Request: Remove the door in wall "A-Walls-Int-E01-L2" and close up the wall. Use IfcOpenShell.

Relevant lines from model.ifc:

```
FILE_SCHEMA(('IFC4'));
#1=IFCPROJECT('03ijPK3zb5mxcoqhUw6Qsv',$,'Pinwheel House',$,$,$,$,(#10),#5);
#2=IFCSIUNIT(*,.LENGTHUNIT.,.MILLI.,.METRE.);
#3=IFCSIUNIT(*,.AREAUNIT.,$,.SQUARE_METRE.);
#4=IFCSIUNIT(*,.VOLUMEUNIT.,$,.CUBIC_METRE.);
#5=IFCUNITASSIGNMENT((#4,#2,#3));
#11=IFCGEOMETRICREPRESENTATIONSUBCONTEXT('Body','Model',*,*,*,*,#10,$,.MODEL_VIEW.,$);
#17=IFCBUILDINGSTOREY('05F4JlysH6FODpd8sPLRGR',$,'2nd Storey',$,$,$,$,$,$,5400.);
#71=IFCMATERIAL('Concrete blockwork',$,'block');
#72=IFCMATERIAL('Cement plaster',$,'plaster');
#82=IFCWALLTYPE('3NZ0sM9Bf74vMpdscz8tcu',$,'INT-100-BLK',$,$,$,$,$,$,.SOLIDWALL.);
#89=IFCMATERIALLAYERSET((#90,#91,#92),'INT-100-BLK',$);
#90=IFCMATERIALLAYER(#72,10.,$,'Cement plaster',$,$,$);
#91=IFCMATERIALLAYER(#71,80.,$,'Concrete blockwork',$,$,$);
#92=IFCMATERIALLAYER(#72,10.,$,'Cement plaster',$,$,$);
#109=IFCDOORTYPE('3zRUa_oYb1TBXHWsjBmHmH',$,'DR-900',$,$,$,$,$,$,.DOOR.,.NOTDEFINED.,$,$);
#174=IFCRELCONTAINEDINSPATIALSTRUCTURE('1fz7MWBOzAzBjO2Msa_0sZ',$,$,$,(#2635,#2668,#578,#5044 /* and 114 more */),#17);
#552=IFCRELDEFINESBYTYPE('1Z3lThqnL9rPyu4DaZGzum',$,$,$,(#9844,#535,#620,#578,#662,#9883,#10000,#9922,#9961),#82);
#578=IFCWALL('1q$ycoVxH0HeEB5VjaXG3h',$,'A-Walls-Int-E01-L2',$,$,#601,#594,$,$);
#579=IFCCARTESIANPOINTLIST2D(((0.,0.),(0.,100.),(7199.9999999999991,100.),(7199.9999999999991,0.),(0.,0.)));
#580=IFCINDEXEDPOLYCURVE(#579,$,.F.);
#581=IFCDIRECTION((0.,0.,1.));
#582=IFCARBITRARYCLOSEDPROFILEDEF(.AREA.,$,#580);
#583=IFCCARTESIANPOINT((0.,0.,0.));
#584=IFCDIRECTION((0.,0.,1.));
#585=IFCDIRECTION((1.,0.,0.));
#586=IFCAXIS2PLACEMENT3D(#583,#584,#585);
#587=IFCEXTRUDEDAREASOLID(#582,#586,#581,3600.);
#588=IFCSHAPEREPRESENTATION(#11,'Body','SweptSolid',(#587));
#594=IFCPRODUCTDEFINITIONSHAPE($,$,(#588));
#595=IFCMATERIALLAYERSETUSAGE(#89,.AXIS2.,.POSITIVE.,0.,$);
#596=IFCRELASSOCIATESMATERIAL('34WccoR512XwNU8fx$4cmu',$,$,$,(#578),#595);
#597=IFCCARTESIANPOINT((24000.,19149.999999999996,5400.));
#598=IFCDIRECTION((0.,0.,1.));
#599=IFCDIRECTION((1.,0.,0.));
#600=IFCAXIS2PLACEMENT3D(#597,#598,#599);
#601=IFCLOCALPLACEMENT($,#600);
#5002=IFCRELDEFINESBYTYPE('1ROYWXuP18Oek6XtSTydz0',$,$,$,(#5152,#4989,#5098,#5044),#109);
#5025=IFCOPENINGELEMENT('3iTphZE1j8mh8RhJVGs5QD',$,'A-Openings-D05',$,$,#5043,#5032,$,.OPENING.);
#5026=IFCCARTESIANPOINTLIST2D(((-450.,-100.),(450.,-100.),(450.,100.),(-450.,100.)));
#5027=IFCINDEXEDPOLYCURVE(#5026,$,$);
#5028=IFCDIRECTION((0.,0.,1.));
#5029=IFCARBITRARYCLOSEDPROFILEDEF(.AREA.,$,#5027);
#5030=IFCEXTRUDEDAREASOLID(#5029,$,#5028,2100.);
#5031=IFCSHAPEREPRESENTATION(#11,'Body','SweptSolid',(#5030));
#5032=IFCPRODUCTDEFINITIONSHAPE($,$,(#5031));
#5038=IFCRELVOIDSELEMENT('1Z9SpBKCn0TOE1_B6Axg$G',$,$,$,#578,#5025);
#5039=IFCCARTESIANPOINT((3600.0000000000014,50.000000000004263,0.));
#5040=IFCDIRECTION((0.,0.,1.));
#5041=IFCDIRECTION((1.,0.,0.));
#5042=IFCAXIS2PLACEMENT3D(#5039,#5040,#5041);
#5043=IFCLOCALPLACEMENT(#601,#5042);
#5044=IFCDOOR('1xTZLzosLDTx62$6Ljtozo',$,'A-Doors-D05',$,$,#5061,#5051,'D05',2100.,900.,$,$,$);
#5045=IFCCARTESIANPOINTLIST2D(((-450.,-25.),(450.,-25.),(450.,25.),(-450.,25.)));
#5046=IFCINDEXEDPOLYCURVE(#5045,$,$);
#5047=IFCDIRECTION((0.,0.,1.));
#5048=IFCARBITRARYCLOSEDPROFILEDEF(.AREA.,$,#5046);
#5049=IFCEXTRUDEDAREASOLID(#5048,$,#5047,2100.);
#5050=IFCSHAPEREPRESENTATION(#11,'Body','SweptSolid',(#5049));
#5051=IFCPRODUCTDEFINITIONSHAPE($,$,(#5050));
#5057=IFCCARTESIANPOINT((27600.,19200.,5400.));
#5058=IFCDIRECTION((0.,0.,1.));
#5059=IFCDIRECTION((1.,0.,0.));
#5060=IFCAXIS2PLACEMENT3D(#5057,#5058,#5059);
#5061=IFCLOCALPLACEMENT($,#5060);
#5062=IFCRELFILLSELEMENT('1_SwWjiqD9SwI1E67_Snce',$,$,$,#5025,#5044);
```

```python
import ifcopenshell
import ifcopenshell.api.feature
import ifcopenshell.api.root
import ifcopenshell.geom
import ifcopenshell.util.shape

model = ifcopenshell.open("model.ifc")
settings = ifcopenshell.geom.settings()


def volume(element):
    """Net volume in cubic metres, openings subtracted."""
    shape = ifcopenshell.geom.create_shape(settings, element)
    return ifcopenshell.util.shape.get_volume(shape.geometry)


door = model.by_id(5044)
opening = door.FillsVoids[0].RelatingOpeningElement
wall = opening.VoidsElements[0].RelatingBuildingElement
before = volume(wall)

ifcopenshell.api.root.remove_product(model, product=door)
ifcopenshell.api.feature.remove_feature(model, feature=opening)

after = volume(wall)

print(f"wall volume {before:.3f} -> {after:.3f} m3")

model.write("model_rev.ifc")
```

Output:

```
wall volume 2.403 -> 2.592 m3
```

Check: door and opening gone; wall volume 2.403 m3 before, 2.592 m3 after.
